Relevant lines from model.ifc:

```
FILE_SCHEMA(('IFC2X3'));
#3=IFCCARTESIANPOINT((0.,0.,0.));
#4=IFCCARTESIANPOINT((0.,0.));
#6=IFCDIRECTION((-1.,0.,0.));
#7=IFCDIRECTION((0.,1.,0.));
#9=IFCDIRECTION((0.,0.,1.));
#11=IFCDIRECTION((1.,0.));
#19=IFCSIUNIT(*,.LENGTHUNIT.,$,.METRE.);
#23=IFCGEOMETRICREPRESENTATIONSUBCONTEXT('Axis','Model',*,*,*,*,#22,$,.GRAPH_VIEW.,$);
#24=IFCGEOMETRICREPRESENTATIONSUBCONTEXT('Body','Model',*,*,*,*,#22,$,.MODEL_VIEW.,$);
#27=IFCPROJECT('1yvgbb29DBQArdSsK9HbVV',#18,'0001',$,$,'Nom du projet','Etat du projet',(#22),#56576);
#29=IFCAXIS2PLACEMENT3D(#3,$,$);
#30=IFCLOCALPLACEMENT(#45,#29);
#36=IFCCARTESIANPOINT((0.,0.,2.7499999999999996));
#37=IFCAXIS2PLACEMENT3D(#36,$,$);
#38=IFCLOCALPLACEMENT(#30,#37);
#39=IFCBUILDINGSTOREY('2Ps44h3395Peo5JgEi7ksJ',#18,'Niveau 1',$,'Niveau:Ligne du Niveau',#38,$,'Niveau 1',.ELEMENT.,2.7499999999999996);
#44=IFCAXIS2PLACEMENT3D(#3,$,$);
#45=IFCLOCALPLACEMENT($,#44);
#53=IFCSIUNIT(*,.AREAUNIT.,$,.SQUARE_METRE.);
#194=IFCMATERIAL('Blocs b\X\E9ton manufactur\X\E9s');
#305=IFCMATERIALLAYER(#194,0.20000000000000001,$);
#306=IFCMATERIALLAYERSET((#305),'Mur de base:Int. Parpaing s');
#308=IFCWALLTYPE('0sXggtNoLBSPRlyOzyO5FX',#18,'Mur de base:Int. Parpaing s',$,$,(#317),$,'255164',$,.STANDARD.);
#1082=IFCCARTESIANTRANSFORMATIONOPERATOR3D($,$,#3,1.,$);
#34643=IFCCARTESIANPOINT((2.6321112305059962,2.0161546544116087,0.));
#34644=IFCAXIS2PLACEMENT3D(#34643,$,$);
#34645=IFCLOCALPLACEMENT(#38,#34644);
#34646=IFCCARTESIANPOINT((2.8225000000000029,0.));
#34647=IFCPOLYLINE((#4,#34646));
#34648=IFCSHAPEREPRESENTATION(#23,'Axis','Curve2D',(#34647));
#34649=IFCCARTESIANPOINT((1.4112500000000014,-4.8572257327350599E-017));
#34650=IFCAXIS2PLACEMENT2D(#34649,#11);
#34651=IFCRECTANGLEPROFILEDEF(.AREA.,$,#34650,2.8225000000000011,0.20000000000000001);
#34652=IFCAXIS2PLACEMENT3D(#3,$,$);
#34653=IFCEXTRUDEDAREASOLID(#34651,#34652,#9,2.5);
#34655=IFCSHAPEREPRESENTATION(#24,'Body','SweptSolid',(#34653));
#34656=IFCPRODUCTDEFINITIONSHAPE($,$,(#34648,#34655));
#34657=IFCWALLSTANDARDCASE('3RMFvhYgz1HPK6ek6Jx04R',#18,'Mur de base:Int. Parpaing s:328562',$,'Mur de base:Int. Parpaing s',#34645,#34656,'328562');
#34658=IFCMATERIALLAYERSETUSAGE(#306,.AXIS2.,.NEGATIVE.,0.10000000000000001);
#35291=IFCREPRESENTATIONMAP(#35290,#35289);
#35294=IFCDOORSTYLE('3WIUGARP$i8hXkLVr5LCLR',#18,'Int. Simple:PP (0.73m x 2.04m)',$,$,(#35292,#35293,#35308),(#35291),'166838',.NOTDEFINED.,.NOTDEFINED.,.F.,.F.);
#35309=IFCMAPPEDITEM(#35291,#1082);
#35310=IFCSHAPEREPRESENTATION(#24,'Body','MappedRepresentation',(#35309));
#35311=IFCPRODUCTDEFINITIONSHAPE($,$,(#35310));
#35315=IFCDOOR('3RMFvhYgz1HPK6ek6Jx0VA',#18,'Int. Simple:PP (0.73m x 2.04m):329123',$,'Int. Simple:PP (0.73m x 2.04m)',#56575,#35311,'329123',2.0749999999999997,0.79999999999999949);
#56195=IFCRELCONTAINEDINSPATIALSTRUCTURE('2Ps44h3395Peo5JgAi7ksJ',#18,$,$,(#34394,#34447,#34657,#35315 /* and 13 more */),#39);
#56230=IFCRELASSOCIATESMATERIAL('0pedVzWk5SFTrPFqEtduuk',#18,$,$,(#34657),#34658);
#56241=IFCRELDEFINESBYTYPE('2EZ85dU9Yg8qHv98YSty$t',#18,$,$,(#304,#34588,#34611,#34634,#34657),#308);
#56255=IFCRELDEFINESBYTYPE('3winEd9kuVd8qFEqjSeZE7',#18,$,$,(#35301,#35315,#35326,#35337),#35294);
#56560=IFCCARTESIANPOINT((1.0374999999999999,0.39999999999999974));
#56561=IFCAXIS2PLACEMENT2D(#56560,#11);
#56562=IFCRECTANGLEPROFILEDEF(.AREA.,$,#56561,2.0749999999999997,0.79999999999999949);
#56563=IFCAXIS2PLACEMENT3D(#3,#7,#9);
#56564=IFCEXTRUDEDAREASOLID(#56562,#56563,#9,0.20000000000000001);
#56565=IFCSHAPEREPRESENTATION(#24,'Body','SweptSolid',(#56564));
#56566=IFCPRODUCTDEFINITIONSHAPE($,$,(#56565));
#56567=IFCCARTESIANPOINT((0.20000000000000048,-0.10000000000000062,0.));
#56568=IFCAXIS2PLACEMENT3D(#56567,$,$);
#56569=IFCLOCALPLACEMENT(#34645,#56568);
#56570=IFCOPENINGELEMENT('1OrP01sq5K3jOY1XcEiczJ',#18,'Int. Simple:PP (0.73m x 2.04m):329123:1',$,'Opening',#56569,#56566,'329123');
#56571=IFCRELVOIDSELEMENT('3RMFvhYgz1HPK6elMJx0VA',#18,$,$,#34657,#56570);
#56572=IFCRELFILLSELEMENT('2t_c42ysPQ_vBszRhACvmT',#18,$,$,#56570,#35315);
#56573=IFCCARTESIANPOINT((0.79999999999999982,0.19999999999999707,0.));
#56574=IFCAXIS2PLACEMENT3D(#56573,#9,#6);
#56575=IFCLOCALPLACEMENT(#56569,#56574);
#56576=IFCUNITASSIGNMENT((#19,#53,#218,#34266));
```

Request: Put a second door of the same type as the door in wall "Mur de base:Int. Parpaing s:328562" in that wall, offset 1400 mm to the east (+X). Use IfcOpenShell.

```python
import ifcopenshell
import ifcopenshell.api.feature
import ifcopenshell.api.geometry
import ifcopenshell.api.root
import ifcopenshell.geom
import ifcopenshell.util.element
import ifcopenshell.util.placement
import ifcopenshell.util.shape

model = ifcopenshell.open("model.ifc")
settings = ifcopenshell.geom.settings()


def volume(element):
    """Net volume in cubic metres, openings subtracted."""
    shape = ifcopenshell.geom.create_shape(settings, element)
    return ifcopenshell.util.shape.get_volume(shape.geometry)


def reuse_history(source, copy):
    """copy_class also copies each property set's owner history, people and application; keep the originals."""
    for rel in copy.IsDefinedBy:
        if rel.is_a("IfcRelDefinesByProperties") and (history := rel.RelatingPropertyDefinition.OwnerHistory):
            rel.RelatingPropertyDefinition.OwnerHistory = source.OwnerHistory
            ifcopenshell.util.element.remove_deep2(model, history)


door = model.by_guid("3RMFvhYgz1HPK6ek6Jx0VA")
opening = door.FillsVoids[0].RelatingOpeningElement
wall = opening.VoidsElements[0].RelatingBuildingElement
before = volume(wall)
shift = ifcopenshell.util.placement.get_local_placement(wall.ObjectPlacement)[:3, 0] * 1.4

# copy_class copies the void relationship, type, container and properties, but no geometry.
new_opening = ifcopenshell.api.root.copy_class(model, product=opening)
new_opening.Representation = ifcopenshell.util.element.copy_deep(
    model, opening.Representation, exclude=["IfcGeometricRepresentationContext", "IfcRepresentationMap"]
)
new_opening.Name = "Int. Simple:PP (0.73m x 2.04m)"
new_opening.Tag = None
new_door = ifcopenshell.api.root.copy_class(model, product=door)
new_door.Representation = ifcopenshell.util.element.copy_deep(
    model, door.Representation, exclude=["IfcGeometricRepresentationContext", "IfcRepresentationMap"]
)
new_door.Name = "Int. Simple:PP (0.73m x 2.04m)"
new_door.Tag = None
reuse_history(door, new_door)
fills = ifcopenshell.api.feature.add_filling(model, opening=new_opening, element=new_door)
fills.OwnerHistory = new_door.OwnerHistory  # required in IFC2X3

for old, new in ((opening, new_opening), (door, new_door)):
    matrix = ifcopenshell.util.placement.get_local_placement(old.ObjectPlacement)
    matrix[:3, 3] += shift
    ifcopenshell.api.geometry.edit_object_placement(model, product=new, matrix=matrix, is_si=False)

after = volume(wall)

print(f"wall volume {before:.3f} -> {after:.3f} m3")

model.write("model_updated.ifc")
```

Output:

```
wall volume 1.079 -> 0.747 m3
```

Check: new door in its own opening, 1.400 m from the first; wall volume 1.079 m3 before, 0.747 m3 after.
